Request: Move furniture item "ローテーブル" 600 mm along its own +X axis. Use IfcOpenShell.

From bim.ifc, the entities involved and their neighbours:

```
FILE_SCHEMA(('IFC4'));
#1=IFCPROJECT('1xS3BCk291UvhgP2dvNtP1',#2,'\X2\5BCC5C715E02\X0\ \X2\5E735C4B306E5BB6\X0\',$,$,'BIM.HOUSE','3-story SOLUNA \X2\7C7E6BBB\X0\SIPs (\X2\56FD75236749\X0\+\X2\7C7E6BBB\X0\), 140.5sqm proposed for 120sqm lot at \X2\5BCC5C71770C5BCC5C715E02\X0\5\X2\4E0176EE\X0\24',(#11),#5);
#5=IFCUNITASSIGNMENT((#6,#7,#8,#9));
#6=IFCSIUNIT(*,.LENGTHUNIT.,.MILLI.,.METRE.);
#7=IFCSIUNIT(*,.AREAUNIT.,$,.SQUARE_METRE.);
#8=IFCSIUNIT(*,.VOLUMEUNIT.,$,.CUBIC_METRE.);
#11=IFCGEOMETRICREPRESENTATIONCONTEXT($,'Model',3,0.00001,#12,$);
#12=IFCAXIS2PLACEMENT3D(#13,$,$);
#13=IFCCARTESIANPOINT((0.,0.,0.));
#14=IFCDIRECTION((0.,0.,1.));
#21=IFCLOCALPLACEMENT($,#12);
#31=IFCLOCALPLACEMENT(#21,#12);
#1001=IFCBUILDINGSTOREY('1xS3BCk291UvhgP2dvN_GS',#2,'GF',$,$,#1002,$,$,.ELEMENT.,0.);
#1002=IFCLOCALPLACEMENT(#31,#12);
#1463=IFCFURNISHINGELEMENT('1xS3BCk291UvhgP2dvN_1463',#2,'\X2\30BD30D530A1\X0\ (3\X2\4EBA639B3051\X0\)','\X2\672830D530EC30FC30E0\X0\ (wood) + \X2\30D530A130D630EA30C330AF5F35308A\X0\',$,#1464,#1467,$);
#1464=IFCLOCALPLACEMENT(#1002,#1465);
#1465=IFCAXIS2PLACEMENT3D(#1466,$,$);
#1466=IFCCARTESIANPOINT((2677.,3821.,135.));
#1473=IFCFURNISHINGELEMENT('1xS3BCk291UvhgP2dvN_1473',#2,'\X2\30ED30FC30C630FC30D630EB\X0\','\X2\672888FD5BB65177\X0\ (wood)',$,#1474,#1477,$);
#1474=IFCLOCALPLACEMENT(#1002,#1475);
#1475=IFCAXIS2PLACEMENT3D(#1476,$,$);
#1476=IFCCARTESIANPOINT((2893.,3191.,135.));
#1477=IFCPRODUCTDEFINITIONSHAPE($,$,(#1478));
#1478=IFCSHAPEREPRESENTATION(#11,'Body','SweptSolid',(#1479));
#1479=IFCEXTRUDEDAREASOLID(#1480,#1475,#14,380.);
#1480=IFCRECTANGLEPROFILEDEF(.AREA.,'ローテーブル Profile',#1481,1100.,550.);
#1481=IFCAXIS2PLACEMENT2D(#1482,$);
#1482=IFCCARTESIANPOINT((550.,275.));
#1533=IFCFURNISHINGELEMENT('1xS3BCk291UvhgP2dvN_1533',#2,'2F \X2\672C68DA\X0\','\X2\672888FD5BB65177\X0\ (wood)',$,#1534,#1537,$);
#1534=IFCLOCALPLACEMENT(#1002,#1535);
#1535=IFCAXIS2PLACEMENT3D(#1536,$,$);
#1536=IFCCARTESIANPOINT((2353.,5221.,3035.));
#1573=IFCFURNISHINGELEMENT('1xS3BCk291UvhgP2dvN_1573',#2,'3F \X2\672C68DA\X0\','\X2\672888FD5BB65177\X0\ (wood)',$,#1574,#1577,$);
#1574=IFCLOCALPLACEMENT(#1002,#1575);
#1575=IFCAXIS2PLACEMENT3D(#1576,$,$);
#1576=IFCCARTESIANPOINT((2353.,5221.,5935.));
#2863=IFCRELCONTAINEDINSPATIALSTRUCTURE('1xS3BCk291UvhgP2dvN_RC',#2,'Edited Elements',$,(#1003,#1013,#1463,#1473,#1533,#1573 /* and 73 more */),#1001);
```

```python
import ifcopenshell
import ifcopenshell.api.geometry
import ifcopenshell.util.placement

model = ifcopenshell.open("bim.ifc")

item = model.by_guid("1xS3BCk291UvhgP2dvN_1473")
matrix = ifcopenshell.util.placement.get_local_placement(item.ObjectPlacement)
matrix[:3, 3] += matrix[:3, 0] * 600.0
ifcopenshell.api.geometry.edit_object_placement(model, product=item, matrix=matrix, is_si=False)

print(ifcopenshell.util.placement.get_local_placement(item.ObjectPlacement).round(3) + 0.0)

model.write("bim_rev.ifc")
```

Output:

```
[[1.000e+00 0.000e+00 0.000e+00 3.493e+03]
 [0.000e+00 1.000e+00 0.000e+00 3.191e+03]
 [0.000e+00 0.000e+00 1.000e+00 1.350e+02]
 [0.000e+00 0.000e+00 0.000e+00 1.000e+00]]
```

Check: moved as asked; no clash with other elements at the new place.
